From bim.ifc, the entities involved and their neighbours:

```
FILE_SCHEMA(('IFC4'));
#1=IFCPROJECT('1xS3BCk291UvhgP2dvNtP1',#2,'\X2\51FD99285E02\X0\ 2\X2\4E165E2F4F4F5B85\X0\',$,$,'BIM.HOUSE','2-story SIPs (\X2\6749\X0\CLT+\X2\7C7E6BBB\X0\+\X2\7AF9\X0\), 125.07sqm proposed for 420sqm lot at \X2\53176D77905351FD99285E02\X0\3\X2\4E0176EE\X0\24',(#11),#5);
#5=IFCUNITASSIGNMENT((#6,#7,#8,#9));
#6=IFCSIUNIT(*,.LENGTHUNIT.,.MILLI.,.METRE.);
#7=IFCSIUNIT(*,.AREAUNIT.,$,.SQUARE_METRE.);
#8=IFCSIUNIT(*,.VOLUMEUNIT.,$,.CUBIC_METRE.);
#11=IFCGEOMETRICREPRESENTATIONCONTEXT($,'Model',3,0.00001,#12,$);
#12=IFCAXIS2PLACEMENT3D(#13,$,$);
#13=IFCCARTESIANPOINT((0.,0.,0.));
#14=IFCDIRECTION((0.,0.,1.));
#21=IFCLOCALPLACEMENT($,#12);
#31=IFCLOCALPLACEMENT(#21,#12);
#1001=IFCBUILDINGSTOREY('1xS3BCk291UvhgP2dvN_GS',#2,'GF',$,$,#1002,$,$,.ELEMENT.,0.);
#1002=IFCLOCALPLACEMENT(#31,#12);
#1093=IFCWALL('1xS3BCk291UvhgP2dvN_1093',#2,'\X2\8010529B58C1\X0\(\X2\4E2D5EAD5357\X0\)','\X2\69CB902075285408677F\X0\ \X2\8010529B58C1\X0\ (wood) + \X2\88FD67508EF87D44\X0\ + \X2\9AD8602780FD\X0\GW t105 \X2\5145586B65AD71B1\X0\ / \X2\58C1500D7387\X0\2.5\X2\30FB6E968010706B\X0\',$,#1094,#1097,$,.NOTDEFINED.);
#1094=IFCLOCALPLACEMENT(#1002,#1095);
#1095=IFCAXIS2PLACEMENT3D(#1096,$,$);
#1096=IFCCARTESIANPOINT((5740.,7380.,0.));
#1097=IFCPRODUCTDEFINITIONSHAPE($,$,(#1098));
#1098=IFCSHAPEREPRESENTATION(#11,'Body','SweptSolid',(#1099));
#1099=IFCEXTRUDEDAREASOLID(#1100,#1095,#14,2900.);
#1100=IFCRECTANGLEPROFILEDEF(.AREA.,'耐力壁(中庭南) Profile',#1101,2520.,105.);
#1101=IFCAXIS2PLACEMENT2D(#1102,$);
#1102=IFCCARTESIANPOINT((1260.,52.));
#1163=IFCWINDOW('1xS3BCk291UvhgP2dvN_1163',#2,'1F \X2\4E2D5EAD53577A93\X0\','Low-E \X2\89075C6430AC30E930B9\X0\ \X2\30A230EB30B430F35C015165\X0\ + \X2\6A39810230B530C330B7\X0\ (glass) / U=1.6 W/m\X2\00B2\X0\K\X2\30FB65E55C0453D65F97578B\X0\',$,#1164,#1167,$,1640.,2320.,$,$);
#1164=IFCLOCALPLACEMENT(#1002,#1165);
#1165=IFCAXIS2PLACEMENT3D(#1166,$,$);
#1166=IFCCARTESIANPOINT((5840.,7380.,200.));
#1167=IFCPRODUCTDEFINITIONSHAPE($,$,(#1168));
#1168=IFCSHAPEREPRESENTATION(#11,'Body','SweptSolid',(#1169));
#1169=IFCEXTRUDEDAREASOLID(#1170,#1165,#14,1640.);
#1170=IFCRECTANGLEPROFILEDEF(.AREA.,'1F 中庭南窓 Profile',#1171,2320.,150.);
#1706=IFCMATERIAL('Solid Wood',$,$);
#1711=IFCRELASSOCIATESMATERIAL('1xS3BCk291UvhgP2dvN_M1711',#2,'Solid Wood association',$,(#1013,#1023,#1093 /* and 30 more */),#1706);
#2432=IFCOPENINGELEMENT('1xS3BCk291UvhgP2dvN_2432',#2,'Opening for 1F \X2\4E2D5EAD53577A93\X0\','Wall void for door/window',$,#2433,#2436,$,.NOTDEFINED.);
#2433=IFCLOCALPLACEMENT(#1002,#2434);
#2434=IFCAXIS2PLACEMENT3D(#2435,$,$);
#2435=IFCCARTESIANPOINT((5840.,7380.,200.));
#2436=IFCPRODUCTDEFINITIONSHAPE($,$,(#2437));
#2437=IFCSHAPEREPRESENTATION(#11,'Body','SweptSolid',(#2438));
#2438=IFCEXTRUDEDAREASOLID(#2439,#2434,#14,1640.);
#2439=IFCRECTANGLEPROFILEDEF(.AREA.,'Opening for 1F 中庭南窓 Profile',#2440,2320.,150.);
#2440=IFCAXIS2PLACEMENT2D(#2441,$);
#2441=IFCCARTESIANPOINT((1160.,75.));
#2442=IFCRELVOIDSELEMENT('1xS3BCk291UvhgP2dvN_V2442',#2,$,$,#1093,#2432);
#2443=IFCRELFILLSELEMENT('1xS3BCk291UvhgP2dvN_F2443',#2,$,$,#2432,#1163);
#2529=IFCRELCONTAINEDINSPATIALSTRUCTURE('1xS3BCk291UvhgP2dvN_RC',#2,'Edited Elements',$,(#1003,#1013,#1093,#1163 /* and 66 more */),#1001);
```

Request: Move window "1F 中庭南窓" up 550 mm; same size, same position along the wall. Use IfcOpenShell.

```python
import numpy as np
import ifcopenshell
import ifcopenshell.api.geometry
import ifcopenshell.util.placement
import ifcopenshell.util.unit

model = ifcopenshell.open("bim.ifc")
unit_scale = ifcopenshell.util.unit.calculate_unit_scale(model)

window = model.by_id(1163)
opening = window.FillsVoids[0].RelatingOpeningElement
dz = 550.0

shift = np.array([0.0, 0.0, dz])
# The window is not placed relative to its opening, so move both.
for product in (opening, window):
    matrix = ifcopenshell.util.placement.get_local_placement(product.ObjectPlacement)
    matrix[:3, 3] += shift
    ifcopenshell.api.geometry.edit_object_placement(model, product=product, matrix=matrix, is_si=False)

print(f"moved by {dz * unit_scale:+.3f} m")

model.write("bim_rev.ifc")
```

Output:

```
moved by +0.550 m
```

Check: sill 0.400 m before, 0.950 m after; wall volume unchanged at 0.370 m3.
